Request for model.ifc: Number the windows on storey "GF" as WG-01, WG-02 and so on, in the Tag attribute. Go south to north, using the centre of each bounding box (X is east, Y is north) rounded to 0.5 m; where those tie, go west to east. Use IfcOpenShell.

First a look at what the model holds.

```python
import ifcopenshell
import ifcopenshell.util.element
import ifcopenshell.util.placement

model = ifcopenshell.open("model.ifc")
print(model.schema)
storey = next(s for s in model.by_type("IfcBuildingStorey") if s.Name == "GF")
windows = [e for e in ifcopenshell.util.element.get_decomposition(storey) if e.is_a("IfcWindow")]
for e in sorted(windows, key=lambda e: e.id()):
    origin = ifcopenshell.util.placement.get_local_placement(e.ObjectPlacement)[:3, 3]
    print(e.id(), e.Tag, e.Name, origin.round(2) + 0.0, sep=" | ")
```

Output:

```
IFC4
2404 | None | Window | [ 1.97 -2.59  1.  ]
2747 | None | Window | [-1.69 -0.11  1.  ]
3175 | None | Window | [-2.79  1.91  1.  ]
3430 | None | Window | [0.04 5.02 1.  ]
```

```python
import ifcopenshell
import ifcopenshell.geom
import ifcopenshell.util.element
import ifcopenshell.util.shape

model = ifcopenshell.open("model.ifc")
settings = ifcopenshell.geom.settings()
settings.set("use-world-coords", True)


def centre(element):
    shape = ifcopenshell.geom.create_shape(settings, element)
    return ifcopenshell.util.shape.get_bbox_centroid(shape.geometry)


storey = next(s for s in model.by_type("IfcBuildingStorey") if s.Name == "GF")
windows = [e for e in ifcopenshell.util.element.get_decomposition(storey) if e.is_a("IfcWindow")]

# Insertion points can sit at a corner or the storey origin, so sort by the geometry (in metres).
centres = {e: centre(e) for e in windows}
windows.sort(key=lambda e: (round(centres[e][1] / 0.5), centres[e][0]))

for i, e in enumerate(windows, start=1):
    number = f"WG-{i:02d}"
    e.Tag = number
    print(e.id(), number)

model.write("model_edited.ifc")
```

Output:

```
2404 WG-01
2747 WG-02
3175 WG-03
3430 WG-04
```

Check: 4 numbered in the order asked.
